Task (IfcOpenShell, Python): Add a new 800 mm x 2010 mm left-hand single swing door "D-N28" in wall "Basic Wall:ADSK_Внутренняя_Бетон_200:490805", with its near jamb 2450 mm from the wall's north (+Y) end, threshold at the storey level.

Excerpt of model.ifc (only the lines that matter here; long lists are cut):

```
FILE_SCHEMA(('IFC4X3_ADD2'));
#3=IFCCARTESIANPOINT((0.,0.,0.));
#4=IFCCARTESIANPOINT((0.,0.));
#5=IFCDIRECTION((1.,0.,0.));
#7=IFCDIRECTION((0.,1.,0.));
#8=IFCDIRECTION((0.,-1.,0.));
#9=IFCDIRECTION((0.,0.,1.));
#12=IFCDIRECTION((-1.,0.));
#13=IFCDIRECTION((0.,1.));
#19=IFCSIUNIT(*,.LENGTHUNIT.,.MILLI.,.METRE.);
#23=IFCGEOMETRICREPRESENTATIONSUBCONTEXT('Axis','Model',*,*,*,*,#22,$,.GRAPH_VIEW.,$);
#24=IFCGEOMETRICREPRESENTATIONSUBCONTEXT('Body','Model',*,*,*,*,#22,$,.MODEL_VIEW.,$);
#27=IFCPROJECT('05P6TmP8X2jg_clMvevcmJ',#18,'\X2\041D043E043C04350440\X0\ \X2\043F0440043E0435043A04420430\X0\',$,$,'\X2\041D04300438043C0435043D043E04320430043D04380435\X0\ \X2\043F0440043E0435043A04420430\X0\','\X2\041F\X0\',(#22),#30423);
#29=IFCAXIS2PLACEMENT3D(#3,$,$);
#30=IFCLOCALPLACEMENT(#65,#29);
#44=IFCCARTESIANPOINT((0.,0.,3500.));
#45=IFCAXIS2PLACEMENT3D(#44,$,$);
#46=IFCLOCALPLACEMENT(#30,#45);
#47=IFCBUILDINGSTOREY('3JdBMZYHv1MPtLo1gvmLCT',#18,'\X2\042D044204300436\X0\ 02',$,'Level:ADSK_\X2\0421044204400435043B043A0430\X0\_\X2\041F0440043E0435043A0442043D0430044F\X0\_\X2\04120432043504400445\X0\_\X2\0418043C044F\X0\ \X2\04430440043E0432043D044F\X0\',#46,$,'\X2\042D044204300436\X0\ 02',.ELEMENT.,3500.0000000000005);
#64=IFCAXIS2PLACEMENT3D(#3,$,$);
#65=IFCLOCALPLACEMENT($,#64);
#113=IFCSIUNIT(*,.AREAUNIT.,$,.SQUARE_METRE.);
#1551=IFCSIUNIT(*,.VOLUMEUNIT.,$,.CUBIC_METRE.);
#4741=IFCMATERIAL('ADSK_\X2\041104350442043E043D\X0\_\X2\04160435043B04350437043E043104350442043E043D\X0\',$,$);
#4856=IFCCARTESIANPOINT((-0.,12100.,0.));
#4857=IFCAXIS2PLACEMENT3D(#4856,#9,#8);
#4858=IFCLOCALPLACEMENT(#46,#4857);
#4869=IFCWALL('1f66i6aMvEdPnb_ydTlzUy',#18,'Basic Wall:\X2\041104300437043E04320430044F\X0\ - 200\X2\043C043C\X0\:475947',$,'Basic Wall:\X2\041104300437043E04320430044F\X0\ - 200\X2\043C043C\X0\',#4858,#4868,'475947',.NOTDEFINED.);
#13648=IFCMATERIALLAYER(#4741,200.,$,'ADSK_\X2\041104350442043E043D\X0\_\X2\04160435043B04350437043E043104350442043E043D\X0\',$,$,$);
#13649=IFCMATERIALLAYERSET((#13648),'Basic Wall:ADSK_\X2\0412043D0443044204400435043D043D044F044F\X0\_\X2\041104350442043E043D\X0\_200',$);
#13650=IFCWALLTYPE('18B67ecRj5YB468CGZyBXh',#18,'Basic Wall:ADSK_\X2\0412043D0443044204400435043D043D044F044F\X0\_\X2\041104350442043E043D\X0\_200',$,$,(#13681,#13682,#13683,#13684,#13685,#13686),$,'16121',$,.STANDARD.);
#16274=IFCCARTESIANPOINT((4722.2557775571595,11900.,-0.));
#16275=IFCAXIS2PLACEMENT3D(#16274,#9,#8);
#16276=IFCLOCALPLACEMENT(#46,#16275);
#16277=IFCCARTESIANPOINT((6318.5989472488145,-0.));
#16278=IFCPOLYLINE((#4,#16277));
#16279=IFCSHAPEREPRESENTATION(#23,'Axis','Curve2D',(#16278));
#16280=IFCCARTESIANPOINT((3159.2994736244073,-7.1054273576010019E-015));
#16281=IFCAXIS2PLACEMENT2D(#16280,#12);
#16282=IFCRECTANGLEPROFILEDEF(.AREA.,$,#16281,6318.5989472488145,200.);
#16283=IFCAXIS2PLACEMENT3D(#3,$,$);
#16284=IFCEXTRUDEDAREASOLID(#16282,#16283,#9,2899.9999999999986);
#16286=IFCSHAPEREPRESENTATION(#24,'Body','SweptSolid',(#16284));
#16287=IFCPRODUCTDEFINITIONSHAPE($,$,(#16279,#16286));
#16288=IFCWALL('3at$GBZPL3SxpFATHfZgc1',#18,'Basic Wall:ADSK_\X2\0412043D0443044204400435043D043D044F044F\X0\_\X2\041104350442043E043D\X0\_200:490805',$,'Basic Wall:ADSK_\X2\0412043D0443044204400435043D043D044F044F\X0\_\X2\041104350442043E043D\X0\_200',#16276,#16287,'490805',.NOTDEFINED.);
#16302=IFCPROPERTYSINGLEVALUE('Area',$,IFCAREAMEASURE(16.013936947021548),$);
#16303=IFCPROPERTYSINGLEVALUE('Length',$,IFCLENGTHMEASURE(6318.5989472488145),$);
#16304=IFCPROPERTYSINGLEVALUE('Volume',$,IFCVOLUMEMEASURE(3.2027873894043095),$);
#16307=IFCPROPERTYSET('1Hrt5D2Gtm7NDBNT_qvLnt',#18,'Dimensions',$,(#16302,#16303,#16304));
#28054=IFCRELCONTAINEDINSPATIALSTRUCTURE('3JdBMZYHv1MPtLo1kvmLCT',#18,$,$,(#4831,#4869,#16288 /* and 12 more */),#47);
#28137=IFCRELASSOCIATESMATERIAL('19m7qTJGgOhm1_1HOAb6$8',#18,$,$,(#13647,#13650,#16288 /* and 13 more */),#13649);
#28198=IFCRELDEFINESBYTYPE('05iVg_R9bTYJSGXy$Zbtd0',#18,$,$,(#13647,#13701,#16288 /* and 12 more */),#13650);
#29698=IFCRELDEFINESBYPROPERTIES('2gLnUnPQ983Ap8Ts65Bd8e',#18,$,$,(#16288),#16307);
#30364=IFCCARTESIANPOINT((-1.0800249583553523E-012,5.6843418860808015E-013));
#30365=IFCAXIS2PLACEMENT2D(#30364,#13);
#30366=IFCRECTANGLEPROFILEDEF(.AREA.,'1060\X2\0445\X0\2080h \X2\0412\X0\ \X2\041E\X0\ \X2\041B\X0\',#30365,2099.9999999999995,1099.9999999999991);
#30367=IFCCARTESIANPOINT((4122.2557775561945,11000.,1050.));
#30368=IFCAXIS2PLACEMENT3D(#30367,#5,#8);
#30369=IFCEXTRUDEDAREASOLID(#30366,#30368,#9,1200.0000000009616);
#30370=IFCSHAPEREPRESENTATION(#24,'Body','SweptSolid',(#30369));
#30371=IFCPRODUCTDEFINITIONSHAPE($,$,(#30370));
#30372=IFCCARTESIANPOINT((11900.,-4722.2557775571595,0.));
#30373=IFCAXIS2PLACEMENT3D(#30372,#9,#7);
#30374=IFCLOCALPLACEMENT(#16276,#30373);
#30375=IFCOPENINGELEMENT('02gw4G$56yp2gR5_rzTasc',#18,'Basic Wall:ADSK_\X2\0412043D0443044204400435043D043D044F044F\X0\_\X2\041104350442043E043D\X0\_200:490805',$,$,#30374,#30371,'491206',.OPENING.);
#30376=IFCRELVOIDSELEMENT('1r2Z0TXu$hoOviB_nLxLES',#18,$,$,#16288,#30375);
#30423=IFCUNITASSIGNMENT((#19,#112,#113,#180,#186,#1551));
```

```python
import numpy as np
import ifcopenshell
import ifcopenshell.api.feature
import ifcopenshell.api.geometry
import ifcopenshell.api.pset
import ifcopenshell.api.root
import ifcopenshell.api.spatial
import ifcopenshell.geom
import ifcopenshell.util.element
import ifcopenshell.util.placement
import ifcopenshell.util.representation
import ifcopenshell.util.shape
import ifcopenshell.util.unit

model = ifcopenshell.open("model.ifc")
unit_scale = ifcopenshell.util.unit.calculate_unit_scale(model)
area_scale = ifcopenshell.util.unit.calculate_unit_scale(model, "AREAUNIT")
volume_scale = ifcopenshell.util.unit.calculate_unit_scale(model, "VOLUMEUNIT")
settings = ifcopenshell.geom.settings()


def volume(element):
    """Net volume in cubic metres, openings subtracted."""
    shape = ifcopenshell.geom.create_shape(settings, element)
    return ifcopenshell.util.shape.get_volume(shape.geometry)


wall = model.by_id(16288)
storey = ifcopenshell.util.element.get_container(wall, ifc_class="IfcBuildingStorey")
context = ifcopenshell.util.representation.get_context(model, "Model", "Body", "MODEL_VIEW")
before = volume(wall)

width, height, from_end, sill = 0.8, 2.01, 2.45, 0.0  # metres

# The wall runs along its own X axis, and the end named is its -X end.
wall_shape = ifcopenshell.geom.create_shape(settings, wall)
x, y, z = ifcopenshell.util.shape.get_vertices(wall_shape.geometry).T
start = x.min() + from_end
face, thickness = float(y.min()), float(y.max() - y.min())
wall_matrix = ifcopenshell.util.placement.get_local_placement(wall.ObjectPlacement)
level = ifcopenshell.util.placement.get_local_placement(storey.ObjectPlacement)[2, 3]


def in_wall(x, y):
    """Placement at x, y metres in the wall's axes, at sill height."""
    matrix = wall_matrix.copy()
    matrix[:, 3] = wall_matrix @ np.array([x / unit_scale, y / unit_scale, 0.0, 1.0])
    matrix[2, 3] = level + sill / unit_scale
    return matrix


# Opening: a box that overshoots both wall faces by 50 mm.
opening = ifcopenshell.api.root.create_entity(model, ifc_class="IfcOpeningElement", predefined_type="OPENING")
box = ifcopenshell.api.geometry.add_wall_representation(
    model, context=context, length=width, height=height, thickness=thickness + 0.1
)
ifcopenshell.api.geometry.assign_representation(model, product=opening, representation=box)
ifcopenshell.api.geometry.edit_object_placement(model, product=opening, matrix=in_wall(start, face - 0.05), is_si=False)
ifcopenshell.api.feature.add_feature(model, feature=opening, element=wall)

door = ifcopenshell.api.root.create_entity(model, ifc_class="IfcDoor", name="D-N28", predefined_type="DOOR")
door.OverallWidth, door.OverallHeight = width / unit_scale, height / unit_scale
door.OperationType = "SINGLE_SWING_LEFT"
body = ifcopenshell.api.geometry.add_door_representation(
    model,
    context=context,
    overall_width=door.OverallWidth,
    overall_height=door.OverallHeight,
    operation_type="SINGLE_SWING_LEFT",
    lining_properties={"LiningDepth": thickness / unit_scale, "ThresholdDepth": thickness / unit_scale},
)
ifcopenshell.api.geometry.assign_representation(model, product=door, representation=body)
ifcopenshell.api.spatial.assign_container(model, products=[door], relating_structure=storey)
ifcopenshell.api.feature.add_filling(model, opening=opening, element=door)

# The lining spans the wall, so the door starts at the wall face.
ifcopenshell.api.geometry.edit_object_placement(model, product=door, matrix=in_wall(start, face), is_si=False)

after = volume(wall)

# Update the wall's stored quantities.
pset = model.by_id(ifcopenshell.util.element.get_pset(wall, "Dimensions", should_inherit=False)["id"])
ifcopenshell.api.pset.edit_pset(model, pset=pset, properties={
    "Area": model.create_entity("IfcAreaMeasure", after / thickness / area_scale),
    "Volume": model.create_entity("IfcVolumeMeasure", after / volume_scale),
})

print(f"wall volume {before:.3f} -> {after:.3f} m3")

model.write("model-out.ifc")
```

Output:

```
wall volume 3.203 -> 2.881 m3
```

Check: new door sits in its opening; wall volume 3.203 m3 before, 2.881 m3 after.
